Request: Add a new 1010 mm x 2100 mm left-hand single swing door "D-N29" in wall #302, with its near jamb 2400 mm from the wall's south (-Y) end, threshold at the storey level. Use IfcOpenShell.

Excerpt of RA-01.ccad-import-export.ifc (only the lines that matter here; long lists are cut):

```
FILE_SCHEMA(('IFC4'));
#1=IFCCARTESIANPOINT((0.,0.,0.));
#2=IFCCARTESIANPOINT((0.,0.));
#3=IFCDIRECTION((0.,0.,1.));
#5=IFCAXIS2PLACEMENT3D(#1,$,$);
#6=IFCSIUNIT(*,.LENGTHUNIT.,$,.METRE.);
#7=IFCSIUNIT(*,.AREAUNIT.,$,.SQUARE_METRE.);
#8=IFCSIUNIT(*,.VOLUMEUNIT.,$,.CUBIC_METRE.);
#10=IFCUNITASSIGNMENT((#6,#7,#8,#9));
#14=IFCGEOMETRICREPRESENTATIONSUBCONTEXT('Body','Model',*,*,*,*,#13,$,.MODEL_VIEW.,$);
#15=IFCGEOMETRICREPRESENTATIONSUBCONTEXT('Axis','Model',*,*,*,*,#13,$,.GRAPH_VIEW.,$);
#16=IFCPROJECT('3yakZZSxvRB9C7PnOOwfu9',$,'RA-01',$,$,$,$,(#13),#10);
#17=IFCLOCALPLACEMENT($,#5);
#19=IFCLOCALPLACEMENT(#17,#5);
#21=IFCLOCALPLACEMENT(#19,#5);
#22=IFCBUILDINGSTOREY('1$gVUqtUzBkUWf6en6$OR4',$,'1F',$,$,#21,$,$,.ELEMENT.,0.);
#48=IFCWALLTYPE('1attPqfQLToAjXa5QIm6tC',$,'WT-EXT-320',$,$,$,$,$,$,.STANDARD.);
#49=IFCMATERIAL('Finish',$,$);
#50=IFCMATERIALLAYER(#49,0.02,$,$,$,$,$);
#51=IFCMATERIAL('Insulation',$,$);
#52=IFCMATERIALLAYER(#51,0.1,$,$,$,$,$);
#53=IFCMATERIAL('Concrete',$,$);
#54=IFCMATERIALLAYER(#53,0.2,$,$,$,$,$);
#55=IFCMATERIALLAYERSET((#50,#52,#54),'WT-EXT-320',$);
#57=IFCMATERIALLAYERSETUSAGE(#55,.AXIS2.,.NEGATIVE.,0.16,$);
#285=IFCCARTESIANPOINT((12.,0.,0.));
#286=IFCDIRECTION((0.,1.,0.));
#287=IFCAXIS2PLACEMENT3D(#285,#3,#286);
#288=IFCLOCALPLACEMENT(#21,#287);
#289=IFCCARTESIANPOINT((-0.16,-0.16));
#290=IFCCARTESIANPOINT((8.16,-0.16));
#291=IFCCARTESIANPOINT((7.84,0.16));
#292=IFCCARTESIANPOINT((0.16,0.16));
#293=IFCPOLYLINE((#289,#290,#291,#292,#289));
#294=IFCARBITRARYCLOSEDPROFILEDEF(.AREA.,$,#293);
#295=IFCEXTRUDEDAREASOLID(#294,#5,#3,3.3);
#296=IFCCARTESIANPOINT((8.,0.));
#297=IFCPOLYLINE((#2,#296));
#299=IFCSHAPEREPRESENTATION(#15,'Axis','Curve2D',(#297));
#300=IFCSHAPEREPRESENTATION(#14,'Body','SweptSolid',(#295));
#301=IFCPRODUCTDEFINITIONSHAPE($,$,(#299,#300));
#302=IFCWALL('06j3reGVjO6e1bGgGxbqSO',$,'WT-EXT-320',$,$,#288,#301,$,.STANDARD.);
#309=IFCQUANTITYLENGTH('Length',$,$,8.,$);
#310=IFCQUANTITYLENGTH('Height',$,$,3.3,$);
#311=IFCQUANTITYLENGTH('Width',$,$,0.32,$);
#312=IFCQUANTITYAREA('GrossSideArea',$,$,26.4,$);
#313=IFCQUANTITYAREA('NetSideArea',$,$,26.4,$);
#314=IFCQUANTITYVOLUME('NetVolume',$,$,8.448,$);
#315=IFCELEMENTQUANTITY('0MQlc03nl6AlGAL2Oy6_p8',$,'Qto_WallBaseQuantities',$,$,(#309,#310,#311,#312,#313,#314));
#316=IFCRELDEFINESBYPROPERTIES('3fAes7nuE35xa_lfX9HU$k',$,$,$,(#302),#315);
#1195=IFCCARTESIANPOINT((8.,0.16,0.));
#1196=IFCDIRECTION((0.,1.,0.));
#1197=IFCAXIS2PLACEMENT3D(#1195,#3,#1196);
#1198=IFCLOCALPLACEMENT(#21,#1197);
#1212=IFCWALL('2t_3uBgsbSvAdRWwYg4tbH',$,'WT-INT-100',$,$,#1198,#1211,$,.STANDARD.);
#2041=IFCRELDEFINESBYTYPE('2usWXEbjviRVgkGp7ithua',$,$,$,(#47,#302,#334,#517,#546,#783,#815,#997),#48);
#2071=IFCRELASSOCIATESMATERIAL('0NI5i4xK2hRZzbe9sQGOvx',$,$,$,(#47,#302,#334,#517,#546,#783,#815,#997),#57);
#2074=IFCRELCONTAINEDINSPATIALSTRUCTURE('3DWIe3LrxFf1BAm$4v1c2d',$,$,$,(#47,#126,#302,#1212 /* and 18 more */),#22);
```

```python
import numpy as np
import ifcopenshell
import ifcopenshell.api.feature
import ifcopenshell.api.geometry
import ifcopenshell.api.pset
import ifcopenshell.api.root
import ifcopenshell.api.spatial
import ifcopenshell.geom
import ifcopenshell.util.element
import ifcopenshell.util.placement
import ifcopenshell.util.representation
import ifcopenshell.util.shape
import ifcopenshell.util.unit

model = ifcopenshell.open("RA-01.ccad-import-export.ifc")
unit_scale = ifcopenshell.util.unit.calculate_unit_scale(model)
area_scale = ifcopenshell.util.unit.calculate_unit_scale(model, "AREAUNIT")
volume_scale = ifcopenshell.util.unit.calculate_unit_scale(model, "VOLUMEUNIT")
settings = ifcopenshell.geom.settings()


def volume(element):
    """Net volume in cubic metres, openings subtracted."""
    shape = ifcopenshell.geom.create_shape(settings, element)
    return ifcopenshell.util.shape.get_volume(shape.geometry)


wall = model.by_guid("06j3reGVjO6e1bGgGxbqSO")
storey = ifcopenshell.util.element.get_container(wall, ifc_class="IfcBuildingStorey")
context = ifcopenshell.util.representation.get_context(model, "Model", "Body", "MODEL_VIEW")
before = volume(wall)

width, height, from_end, sill = 1.01, 2.1, 2.4, 0.0  # metres

# The wall runs along its own X axis, and the end named is its -X end.
wall_shape = ifcopenshell.geom.create_shape(settings, wall)
x, y, z = ifcopenshell.util.shape.get_vertices(wall_shape.geometry).T
start = x.min() + from_end
face, thickness = float(y.min()), float(y.max() - y.min())
wall_matrix = ifcopenshell.util.placement.get_local_placement(wall.ObjectPlacement)
level = ifcopenshell.util.placement.get_local_placement(storey.ObjectPlacement)[2, 3]


def in_wall(x, y):
    """Placement at x, y metres in the wall's axes, at sill height."""
    matrix = wall_matrix.copy()
    matrix[:, 3] = wall_matrix @ np.array([x / unit_scale, y / unit_scale, 0.0, 1.0])
    matrix[2, 3] = level + sill / unit_scale
    return matrix


# Opening: a box that overshoots both wall faces by 50 mm.
opening = ifcopenshell.api.root.create_entity(model, ifc_class="IfcOpeningElement", predefined_type="OPENING")
box = ifcopenshell.api.geometry.add_wall_representation(
    model, context=context, length=width, height=height, thickness=thickness + 0.1
)
ifcopenshell.api.geometry.assign_representation(model, product=opening, representation=box)
ifcopenshell.api.geometry.edit_object_placement(model, product=opening, matrix=in_wall(start, face - 0.05), is_si=False)
ifcopenshell.api.feature.add_feature(model, feature=opening, element=wall)

door = ifcopenshell.api.root.create_entity(model, ifc_class="IfcDoor", name="D-N29", predefined_type="DOOR")
door.OverallWidth, door.OverallHeight = width / unit_scale, height / unit_scale
door.OperationType = "SINGLE_SWING_LEFT"
body = ifcopenshell.api.geometry.add_door_representation(
    model,
    context=context,
    overall_width=door.OverallWidth,
    overall_height=door.OverallHeight,
    operation_type="SINGLE_SWING_LEFT",
    lining_properties={"LiningDepth": thickness / unit_scale, "ThresholdDepth": thickness / unit_scale},
)
ifcopenshell.api.geometry.assign_representation(model, product=door, representation=body)
ifcopenshell.api.spatial.assign_container(model, products=[door], relating_structure=storey)
ifcopenshell.api.feature.add_filling(model, opening=opening, element=door)

# The lining spans the wall, so the door starts at the wall face.
ifcopenshell.api.geometry.edit_object_placement(model, product=door, matrix=in_wall(start, face), is_si=False)

after = volume(wall)

# Update the wall's stored quantities.
qto = model.by_id(ifcopenshell.util.element.get_pset(wall, "Qto_WallBaseQuantities", should_inherit=False)["id"])
ifcopenshell.api.pset.edit_qto(model, qto=qto, properties={
    "NetSideArea": after / thickness / area_scale,
    "NetVolume": after / volume_scale,
})

print(f"wall volume {before:.3f} -> {after:.3f} m3")

model.write("RA-01.ccad-import-export_edited.ifc")
```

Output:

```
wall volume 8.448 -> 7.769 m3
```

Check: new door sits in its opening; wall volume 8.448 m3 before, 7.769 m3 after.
